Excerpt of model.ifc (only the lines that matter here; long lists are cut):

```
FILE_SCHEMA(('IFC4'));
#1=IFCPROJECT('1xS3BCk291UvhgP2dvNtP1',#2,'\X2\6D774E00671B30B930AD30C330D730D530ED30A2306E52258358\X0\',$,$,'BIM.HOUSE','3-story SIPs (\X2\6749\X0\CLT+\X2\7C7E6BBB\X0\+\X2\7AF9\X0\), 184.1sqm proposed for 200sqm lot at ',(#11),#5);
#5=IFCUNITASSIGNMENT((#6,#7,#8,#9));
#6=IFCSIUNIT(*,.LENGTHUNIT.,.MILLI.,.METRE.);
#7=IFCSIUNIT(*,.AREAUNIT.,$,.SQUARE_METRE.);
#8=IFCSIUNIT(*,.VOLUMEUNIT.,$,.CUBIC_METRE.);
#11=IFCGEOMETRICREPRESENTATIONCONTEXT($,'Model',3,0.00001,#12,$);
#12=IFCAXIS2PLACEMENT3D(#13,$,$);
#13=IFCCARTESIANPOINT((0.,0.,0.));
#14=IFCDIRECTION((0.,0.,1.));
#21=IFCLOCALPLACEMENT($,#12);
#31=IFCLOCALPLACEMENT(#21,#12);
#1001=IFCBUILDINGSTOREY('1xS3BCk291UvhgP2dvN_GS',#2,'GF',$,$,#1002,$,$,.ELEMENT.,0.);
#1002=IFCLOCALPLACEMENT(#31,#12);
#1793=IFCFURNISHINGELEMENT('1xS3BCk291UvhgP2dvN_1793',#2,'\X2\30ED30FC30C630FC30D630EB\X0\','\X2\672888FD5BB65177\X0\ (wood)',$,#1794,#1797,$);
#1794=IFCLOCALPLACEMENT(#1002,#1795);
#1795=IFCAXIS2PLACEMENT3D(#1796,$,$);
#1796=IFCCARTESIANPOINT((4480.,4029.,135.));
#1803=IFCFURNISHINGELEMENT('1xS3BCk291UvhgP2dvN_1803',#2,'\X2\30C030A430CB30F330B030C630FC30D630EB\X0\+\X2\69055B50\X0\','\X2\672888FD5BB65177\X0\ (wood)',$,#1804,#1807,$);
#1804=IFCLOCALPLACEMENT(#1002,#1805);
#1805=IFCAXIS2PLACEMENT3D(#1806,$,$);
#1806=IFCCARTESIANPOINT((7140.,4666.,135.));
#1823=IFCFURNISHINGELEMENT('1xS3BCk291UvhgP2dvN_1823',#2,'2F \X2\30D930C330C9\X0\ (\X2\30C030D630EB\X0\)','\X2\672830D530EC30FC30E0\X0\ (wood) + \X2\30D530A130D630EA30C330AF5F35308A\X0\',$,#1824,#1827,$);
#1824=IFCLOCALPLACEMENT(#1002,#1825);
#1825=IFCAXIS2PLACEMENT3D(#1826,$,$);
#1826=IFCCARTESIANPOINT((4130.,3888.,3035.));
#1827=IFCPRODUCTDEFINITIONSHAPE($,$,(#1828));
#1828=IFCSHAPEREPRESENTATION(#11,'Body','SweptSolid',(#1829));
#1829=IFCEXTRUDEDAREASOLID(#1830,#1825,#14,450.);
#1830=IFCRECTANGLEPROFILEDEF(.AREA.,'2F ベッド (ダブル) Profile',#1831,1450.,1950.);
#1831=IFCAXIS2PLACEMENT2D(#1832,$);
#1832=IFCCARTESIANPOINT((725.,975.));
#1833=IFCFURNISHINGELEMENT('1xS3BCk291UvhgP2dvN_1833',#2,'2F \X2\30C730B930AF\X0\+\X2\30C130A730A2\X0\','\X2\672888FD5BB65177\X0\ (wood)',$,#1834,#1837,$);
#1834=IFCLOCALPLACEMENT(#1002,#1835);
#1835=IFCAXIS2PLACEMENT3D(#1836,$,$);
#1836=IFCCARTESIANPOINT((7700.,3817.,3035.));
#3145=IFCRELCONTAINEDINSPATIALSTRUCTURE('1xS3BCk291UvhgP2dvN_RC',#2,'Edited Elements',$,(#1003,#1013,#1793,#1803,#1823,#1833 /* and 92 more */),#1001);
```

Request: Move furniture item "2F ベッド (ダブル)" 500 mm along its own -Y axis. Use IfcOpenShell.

```python
import ifcopenshell
import ifcopenshell.api.geometry
import ifcopenshell.util.placement

model = ifcopenshell.open("model.ifc")

item = model.by_guid("1xS3BCk291UvhgP2dvN_1823")
matrix = ifcopenshell.util.placement.get_local_placement(item.ObjectPlacement)
matrix[:3, 3] -= matrix[:3, 1] * 500.0
ifcopenshell.api.geometry.edit_object_placement(model, product=item, matrix=matrix, is_si=False)

print(ifcopenshell.util.placement.get_local_placement(item.ObjectPlacement).round(3) + 0.0)

model.write("model_edited.ifc")
```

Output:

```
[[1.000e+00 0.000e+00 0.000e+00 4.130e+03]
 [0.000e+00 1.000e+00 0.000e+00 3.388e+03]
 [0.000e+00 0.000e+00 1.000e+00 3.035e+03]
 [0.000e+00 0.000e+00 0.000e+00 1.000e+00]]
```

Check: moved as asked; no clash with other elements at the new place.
